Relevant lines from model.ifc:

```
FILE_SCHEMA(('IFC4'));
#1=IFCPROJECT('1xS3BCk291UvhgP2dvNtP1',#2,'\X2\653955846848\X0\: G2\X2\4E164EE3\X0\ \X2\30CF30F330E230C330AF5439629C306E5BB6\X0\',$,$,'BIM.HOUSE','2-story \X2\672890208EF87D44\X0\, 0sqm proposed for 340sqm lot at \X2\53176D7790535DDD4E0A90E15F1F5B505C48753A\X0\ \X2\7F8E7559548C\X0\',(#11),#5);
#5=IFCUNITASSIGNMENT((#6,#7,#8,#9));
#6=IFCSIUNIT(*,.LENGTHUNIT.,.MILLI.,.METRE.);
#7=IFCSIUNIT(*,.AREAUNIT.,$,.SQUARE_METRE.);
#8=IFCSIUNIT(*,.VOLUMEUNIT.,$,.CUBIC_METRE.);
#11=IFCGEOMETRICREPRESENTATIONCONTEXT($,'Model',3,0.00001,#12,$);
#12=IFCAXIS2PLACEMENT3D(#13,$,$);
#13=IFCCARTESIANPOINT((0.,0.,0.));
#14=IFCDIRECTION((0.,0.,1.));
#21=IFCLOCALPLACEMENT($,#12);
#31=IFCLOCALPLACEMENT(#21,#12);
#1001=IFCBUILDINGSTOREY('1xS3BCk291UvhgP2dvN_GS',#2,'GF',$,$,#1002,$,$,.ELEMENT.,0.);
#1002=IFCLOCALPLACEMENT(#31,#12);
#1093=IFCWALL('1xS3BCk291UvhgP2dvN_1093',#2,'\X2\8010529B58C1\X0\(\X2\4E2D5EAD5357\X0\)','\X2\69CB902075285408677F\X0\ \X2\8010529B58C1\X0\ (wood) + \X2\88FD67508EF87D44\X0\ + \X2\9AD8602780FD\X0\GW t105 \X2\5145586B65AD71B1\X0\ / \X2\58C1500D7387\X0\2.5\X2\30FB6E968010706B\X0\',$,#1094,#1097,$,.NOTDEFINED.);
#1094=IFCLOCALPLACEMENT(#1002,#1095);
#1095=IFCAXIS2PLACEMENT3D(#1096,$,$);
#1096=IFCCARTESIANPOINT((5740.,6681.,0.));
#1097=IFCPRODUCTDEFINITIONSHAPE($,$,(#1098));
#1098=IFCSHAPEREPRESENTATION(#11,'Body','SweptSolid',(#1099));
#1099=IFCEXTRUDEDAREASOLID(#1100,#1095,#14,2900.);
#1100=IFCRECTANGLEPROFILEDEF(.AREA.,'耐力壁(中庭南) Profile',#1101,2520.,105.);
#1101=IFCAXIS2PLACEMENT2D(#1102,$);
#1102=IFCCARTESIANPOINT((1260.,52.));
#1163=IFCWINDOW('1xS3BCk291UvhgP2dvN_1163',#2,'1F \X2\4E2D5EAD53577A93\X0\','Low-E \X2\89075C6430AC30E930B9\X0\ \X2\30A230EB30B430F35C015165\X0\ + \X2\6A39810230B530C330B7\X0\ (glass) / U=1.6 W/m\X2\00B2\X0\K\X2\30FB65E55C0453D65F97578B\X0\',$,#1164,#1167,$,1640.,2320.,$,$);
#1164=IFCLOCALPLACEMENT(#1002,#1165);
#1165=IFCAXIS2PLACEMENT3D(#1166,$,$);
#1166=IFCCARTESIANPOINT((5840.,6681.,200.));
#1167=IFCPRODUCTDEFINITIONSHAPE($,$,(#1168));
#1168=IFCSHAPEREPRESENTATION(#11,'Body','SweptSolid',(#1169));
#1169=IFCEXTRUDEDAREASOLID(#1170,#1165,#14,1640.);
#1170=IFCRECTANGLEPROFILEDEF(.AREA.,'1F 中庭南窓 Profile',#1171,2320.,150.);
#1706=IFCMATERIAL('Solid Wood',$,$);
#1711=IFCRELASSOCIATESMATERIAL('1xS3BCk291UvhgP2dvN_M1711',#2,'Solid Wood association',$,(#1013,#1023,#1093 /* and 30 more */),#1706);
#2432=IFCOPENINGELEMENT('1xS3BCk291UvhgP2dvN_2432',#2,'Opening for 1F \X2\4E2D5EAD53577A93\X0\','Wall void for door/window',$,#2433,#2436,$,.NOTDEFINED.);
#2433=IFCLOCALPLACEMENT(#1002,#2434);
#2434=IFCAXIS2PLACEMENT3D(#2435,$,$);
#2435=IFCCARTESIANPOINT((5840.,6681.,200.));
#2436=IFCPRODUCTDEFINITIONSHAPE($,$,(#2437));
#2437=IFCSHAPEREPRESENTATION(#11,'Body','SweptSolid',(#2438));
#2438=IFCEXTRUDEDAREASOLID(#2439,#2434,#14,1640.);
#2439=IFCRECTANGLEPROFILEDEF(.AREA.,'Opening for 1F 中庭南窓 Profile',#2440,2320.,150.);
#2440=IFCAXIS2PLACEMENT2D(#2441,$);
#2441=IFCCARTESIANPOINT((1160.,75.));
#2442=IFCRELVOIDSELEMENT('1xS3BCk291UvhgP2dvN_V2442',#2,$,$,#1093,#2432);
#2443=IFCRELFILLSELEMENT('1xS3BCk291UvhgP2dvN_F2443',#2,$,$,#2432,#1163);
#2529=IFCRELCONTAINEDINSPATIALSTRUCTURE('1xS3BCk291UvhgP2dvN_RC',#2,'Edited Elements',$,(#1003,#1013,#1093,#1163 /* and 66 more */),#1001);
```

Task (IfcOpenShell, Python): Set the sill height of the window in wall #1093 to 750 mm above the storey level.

```python
import numpy as np
import ifcopenshell
import ifcopenshell.api.geometry
import ifcopenshell.geom
import ifcopenshell.util.element
import ifcopenshell.util.placement
import ifcopenshell.util.shape
import ifcopenshell.util.unit

model = ifcopenshell.open("model.ifc")
unit_scale = ifcopenshell.util.unit.calculate_unit_scale(model)

window = model.by_id(1163)
opening = window.FillsVoids[0].RelatingOpeningElement
storey = ifcopenshell.util.element.get_container(window, ifc_class="IfcBuildingStorey")
level = ifcopenshell.util.placement.get_local_placement(storey.ObjectPlacement)[2, 3]

# The opening's origin need not be at the sill, so measure its lowest point.
shape = ifcopenshell.geom.create_shape(ifcopenshell.geom.settings(), opening)
bottom = ifcopenshell.util.shape.get_shape_bottom_elevation(shape, shape.geometry) / unit_scale
dz = level + 750.0 - bottom

shift = np.array([0.0, 0.0, dz])
# The window is not placed relative to its opening, so move both.
for product in (opening, window):
    matrix = ifcopenshell.util.placement.get_local_placement(product.ObjectPlacement)
    matrix[:3, 3] += shift
    ifcopenshell.api.geometry.edit_object_placement(model, product=product, matrix=matrix, is_si=False)

print(f"moved by {dz * unit_scale:+.3f} m")

model.write("model_updated.ifc")
```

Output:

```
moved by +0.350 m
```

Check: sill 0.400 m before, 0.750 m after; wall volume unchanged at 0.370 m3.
